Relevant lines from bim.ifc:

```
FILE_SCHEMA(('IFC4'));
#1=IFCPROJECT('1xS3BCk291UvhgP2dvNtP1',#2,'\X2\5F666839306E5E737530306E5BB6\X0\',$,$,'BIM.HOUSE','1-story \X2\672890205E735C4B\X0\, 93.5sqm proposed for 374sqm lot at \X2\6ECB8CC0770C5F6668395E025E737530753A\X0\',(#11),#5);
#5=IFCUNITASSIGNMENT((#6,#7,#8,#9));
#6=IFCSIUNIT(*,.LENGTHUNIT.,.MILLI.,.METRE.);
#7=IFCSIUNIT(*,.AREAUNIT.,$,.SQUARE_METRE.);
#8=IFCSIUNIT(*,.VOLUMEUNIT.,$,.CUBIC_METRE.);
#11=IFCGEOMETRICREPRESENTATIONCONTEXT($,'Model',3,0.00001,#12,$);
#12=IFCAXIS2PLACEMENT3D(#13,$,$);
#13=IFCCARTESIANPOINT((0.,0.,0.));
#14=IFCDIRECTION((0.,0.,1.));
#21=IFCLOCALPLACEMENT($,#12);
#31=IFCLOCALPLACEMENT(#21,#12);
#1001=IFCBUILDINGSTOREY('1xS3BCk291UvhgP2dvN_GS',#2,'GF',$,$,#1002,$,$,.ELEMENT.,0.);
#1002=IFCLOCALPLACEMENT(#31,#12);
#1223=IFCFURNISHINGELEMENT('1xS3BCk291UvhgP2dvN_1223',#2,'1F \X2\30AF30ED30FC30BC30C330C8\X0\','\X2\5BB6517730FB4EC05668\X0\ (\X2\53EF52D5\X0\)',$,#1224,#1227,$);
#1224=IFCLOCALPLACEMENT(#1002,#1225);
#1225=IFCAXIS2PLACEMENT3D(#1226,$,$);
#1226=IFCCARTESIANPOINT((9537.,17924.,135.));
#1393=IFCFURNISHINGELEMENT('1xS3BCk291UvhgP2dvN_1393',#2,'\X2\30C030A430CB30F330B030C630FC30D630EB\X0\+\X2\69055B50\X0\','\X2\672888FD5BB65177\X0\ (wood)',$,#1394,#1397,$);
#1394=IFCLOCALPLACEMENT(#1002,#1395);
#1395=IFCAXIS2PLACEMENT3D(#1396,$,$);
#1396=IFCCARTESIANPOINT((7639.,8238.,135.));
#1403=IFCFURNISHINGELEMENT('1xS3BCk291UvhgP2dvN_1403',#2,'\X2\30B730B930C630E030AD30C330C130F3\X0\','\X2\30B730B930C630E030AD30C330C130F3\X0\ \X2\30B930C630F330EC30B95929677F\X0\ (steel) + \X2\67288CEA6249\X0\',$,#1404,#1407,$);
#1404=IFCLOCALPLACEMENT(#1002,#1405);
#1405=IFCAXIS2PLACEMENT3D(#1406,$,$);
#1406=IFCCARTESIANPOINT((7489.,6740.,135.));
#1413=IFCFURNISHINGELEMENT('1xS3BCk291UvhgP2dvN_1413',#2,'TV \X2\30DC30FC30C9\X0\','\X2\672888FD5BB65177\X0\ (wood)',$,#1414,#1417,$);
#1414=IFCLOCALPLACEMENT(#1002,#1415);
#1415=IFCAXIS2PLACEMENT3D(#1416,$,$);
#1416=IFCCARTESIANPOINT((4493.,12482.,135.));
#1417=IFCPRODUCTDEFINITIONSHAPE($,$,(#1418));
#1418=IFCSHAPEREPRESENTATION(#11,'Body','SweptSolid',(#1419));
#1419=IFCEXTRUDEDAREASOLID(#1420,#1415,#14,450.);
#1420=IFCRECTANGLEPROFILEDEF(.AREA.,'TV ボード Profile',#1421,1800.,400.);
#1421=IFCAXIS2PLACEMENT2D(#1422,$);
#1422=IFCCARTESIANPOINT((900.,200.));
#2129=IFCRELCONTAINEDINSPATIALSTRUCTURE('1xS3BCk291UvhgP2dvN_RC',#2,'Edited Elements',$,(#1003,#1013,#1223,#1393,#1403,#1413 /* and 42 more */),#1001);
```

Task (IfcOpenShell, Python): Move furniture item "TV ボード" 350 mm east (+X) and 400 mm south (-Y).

```python
import ifcopenshell
import ifcopenshell.api.geometry
import ifcopenshell.util.placement
import ifcopenshell.util.unit

model = ifcopenshell.open("bim.ifc")
unit_scale = ifcopenshell.util.unit.calculate_unit_scale(model)

item = model.by_id(1413)
matrix = ifcopenshell.util.placement.get_local_placement(item.ObjectPlacement)
matrix[0, 3] += 0.35 / unit_scale
matrix[1, 3] -= 0.4 / unit_scale
ifcopenshell.api.geometry.edit_object_placement(model, product=item, matrix=matrix, is_si=False)

print(ifcopenshell.util.placement.get_local_placement(item.ObjectPlacement).round(3) + 0.0)

model.write("bim_v2.ifc")
```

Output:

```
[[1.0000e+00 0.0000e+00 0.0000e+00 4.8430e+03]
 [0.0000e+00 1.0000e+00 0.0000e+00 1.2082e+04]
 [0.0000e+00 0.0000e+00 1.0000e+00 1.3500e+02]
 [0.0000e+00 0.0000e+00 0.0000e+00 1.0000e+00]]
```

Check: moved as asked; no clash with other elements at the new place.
